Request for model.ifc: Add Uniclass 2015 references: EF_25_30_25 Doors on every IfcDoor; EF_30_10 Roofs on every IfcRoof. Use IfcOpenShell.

First a look at what the model holds.

```python
import ifcopenshell

model = ifcopenshell.open("model.ifc")
print(model.schema)
print("classifications:", [c.Name for c in model.by_type("IfcClassification")])
for ifc_class in ("IfcDoor", "IfcRoof", "IfcStair", "IfcWall", "IfcWindow"):
    print(ifc_class, len(model.by_type(ifc_class)))
```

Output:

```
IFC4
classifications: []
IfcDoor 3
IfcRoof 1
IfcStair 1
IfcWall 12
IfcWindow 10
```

```python
import ifcopenshell
import ifcopenshell.api.classification

model = ifcopenshell.open("model.ifc")

system = ifcopenshell.api.classification.add_classification(model, classification="Uniclass 2015")

codes = {
    "IfcDoor": ("EF_25_30_25", "Doors"),
    "IfcRoof": ("EF_30_10", "Roofs"),
}
for ifc_class, (code, name) in codes.items():
    products = model.by_type(ifc_class)
    ifcopenshell.api.classification.add_reference(
        model, products=products, classification=system, identification=code, name=name
    )
    print(code, len(products))

model.write("model_edited.ifc")
```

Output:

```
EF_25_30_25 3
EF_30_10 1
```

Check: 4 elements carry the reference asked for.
